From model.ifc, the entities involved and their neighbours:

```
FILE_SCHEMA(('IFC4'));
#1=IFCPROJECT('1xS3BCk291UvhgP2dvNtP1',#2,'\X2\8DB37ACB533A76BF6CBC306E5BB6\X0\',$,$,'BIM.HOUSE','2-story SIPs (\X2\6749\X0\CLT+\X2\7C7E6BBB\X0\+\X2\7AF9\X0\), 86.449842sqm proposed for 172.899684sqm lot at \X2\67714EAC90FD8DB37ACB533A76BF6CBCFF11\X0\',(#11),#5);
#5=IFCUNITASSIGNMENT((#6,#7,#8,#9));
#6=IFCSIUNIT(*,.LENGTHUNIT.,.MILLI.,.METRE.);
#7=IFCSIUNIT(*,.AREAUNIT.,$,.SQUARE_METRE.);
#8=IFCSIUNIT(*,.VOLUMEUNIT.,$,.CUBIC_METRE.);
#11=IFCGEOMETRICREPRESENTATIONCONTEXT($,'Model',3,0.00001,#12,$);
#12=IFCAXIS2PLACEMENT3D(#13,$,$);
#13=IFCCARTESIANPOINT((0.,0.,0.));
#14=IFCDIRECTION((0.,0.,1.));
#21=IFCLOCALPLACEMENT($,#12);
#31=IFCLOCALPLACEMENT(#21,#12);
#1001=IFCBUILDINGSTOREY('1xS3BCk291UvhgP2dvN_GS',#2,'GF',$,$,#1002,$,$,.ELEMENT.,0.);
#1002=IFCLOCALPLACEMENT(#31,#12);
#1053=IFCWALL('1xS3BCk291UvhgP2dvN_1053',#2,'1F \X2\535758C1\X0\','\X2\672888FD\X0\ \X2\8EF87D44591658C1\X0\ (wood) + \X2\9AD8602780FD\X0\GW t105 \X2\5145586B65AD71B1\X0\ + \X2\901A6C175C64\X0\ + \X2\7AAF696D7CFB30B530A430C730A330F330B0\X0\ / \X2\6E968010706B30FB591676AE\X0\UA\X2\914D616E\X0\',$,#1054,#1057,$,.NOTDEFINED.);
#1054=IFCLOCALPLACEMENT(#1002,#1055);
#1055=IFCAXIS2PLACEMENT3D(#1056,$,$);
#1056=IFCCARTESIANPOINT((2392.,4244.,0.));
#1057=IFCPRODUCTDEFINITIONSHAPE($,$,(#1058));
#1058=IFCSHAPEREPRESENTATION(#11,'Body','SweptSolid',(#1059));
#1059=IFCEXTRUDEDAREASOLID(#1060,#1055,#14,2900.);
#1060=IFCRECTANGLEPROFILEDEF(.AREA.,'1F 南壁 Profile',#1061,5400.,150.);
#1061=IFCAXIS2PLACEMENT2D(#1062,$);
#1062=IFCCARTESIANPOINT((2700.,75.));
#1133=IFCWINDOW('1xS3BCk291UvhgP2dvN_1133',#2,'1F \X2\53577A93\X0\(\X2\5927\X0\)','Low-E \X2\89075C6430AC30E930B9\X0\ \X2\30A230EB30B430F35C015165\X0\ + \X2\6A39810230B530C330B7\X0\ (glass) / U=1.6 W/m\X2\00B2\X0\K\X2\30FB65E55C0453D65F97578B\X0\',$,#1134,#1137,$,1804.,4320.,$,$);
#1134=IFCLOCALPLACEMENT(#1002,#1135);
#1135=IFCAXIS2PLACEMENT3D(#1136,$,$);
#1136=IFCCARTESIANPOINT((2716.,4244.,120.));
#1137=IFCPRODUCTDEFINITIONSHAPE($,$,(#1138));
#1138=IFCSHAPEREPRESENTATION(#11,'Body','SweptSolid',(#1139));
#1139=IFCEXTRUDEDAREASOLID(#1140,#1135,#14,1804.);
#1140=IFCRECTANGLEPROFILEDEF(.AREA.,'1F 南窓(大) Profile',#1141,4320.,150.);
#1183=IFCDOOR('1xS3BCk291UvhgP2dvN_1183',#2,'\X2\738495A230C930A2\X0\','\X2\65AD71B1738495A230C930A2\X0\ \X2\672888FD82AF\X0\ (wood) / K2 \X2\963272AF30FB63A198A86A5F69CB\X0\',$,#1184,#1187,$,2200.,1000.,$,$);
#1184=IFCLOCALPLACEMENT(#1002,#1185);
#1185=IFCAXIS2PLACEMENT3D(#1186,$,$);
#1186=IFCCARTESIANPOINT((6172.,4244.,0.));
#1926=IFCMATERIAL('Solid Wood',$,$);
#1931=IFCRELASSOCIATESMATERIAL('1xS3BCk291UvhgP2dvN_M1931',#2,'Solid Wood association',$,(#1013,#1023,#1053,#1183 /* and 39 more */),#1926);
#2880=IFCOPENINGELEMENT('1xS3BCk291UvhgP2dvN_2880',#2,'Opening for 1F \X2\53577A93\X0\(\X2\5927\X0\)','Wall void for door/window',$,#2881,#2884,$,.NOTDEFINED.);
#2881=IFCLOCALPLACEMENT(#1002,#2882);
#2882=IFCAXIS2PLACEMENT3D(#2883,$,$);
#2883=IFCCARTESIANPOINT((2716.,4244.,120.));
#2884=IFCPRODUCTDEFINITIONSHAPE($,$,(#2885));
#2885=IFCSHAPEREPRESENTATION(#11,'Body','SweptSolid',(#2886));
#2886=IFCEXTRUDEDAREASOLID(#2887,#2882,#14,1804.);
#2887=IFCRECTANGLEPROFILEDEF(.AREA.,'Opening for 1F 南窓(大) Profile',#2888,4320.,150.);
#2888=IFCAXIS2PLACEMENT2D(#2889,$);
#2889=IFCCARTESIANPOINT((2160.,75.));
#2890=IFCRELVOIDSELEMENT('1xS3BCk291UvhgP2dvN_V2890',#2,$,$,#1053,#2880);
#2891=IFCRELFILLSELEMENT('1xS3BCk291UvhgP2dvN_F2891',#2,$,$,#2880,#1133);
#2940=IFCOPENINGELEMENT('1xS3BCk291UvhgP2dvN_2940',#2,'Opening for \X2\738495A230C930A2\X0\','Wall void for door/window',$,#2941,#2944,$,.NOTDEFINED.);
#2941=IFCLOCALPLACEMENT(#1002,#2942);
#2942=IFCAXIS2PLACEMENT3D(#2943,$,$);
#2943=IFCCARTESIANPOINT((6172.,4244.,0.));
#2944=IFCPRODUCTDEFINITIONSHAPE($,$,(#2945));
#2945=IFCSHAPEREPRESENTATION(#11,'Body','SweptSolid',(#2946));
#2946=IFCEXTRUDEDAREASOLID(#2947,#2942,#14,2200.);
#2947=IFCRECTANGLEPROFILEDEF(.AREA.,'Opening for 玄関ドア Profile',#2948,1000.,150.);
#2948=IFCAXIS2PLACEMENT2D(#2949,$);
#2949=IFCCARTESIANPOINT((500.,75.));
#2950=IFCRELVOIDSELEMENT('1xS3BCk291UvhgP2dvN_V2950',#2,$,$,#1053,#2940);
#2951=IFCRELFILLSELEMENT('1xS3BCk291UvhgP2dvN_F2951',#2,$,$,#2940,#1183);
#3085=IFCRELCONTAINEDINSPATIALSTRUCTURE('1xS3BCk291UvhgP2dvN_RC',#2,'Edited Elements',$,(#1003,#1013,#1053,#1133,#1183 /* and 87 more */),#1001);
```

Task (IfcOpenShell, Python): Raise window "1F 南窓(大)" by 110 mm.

```python
import numpy as np
import ifcopenshell
import ifcopenshell.api.geometry
import ifcopenshell.util.placement
import ifcopenshell.util.unit

model = ifcopenshell.open("model.ifc")
unit_scale = ifcopenshell.util.unit.calculate_unit_scale(model)

window = model.by_guid("1xS3BCk291UvhgP2dvN_1133")
opening = window.FillsVoids[0].RelatingOpeningElement
dz = 0.11 / unit_scale

shift = np.array([0.0, 0.0, dz])
# The window is not placed relative to its opening, so move both.
for product in (opening, window):
    matrix = ifcopenshell.util.placement.get_local_placement(product.ObjectPlacement)
    matrix[:3, 3] += shift
    ifcopenshell.api.geometry.edit_object_placement(model, product=product, matrix=matrix, is_si=False)

print(f"moved by {dz * unit_scale:+.3f} m")

model.write("model_edited.ifc")
```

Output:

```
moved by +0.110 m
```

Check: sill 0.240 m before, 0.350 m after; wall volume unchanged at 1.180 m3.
